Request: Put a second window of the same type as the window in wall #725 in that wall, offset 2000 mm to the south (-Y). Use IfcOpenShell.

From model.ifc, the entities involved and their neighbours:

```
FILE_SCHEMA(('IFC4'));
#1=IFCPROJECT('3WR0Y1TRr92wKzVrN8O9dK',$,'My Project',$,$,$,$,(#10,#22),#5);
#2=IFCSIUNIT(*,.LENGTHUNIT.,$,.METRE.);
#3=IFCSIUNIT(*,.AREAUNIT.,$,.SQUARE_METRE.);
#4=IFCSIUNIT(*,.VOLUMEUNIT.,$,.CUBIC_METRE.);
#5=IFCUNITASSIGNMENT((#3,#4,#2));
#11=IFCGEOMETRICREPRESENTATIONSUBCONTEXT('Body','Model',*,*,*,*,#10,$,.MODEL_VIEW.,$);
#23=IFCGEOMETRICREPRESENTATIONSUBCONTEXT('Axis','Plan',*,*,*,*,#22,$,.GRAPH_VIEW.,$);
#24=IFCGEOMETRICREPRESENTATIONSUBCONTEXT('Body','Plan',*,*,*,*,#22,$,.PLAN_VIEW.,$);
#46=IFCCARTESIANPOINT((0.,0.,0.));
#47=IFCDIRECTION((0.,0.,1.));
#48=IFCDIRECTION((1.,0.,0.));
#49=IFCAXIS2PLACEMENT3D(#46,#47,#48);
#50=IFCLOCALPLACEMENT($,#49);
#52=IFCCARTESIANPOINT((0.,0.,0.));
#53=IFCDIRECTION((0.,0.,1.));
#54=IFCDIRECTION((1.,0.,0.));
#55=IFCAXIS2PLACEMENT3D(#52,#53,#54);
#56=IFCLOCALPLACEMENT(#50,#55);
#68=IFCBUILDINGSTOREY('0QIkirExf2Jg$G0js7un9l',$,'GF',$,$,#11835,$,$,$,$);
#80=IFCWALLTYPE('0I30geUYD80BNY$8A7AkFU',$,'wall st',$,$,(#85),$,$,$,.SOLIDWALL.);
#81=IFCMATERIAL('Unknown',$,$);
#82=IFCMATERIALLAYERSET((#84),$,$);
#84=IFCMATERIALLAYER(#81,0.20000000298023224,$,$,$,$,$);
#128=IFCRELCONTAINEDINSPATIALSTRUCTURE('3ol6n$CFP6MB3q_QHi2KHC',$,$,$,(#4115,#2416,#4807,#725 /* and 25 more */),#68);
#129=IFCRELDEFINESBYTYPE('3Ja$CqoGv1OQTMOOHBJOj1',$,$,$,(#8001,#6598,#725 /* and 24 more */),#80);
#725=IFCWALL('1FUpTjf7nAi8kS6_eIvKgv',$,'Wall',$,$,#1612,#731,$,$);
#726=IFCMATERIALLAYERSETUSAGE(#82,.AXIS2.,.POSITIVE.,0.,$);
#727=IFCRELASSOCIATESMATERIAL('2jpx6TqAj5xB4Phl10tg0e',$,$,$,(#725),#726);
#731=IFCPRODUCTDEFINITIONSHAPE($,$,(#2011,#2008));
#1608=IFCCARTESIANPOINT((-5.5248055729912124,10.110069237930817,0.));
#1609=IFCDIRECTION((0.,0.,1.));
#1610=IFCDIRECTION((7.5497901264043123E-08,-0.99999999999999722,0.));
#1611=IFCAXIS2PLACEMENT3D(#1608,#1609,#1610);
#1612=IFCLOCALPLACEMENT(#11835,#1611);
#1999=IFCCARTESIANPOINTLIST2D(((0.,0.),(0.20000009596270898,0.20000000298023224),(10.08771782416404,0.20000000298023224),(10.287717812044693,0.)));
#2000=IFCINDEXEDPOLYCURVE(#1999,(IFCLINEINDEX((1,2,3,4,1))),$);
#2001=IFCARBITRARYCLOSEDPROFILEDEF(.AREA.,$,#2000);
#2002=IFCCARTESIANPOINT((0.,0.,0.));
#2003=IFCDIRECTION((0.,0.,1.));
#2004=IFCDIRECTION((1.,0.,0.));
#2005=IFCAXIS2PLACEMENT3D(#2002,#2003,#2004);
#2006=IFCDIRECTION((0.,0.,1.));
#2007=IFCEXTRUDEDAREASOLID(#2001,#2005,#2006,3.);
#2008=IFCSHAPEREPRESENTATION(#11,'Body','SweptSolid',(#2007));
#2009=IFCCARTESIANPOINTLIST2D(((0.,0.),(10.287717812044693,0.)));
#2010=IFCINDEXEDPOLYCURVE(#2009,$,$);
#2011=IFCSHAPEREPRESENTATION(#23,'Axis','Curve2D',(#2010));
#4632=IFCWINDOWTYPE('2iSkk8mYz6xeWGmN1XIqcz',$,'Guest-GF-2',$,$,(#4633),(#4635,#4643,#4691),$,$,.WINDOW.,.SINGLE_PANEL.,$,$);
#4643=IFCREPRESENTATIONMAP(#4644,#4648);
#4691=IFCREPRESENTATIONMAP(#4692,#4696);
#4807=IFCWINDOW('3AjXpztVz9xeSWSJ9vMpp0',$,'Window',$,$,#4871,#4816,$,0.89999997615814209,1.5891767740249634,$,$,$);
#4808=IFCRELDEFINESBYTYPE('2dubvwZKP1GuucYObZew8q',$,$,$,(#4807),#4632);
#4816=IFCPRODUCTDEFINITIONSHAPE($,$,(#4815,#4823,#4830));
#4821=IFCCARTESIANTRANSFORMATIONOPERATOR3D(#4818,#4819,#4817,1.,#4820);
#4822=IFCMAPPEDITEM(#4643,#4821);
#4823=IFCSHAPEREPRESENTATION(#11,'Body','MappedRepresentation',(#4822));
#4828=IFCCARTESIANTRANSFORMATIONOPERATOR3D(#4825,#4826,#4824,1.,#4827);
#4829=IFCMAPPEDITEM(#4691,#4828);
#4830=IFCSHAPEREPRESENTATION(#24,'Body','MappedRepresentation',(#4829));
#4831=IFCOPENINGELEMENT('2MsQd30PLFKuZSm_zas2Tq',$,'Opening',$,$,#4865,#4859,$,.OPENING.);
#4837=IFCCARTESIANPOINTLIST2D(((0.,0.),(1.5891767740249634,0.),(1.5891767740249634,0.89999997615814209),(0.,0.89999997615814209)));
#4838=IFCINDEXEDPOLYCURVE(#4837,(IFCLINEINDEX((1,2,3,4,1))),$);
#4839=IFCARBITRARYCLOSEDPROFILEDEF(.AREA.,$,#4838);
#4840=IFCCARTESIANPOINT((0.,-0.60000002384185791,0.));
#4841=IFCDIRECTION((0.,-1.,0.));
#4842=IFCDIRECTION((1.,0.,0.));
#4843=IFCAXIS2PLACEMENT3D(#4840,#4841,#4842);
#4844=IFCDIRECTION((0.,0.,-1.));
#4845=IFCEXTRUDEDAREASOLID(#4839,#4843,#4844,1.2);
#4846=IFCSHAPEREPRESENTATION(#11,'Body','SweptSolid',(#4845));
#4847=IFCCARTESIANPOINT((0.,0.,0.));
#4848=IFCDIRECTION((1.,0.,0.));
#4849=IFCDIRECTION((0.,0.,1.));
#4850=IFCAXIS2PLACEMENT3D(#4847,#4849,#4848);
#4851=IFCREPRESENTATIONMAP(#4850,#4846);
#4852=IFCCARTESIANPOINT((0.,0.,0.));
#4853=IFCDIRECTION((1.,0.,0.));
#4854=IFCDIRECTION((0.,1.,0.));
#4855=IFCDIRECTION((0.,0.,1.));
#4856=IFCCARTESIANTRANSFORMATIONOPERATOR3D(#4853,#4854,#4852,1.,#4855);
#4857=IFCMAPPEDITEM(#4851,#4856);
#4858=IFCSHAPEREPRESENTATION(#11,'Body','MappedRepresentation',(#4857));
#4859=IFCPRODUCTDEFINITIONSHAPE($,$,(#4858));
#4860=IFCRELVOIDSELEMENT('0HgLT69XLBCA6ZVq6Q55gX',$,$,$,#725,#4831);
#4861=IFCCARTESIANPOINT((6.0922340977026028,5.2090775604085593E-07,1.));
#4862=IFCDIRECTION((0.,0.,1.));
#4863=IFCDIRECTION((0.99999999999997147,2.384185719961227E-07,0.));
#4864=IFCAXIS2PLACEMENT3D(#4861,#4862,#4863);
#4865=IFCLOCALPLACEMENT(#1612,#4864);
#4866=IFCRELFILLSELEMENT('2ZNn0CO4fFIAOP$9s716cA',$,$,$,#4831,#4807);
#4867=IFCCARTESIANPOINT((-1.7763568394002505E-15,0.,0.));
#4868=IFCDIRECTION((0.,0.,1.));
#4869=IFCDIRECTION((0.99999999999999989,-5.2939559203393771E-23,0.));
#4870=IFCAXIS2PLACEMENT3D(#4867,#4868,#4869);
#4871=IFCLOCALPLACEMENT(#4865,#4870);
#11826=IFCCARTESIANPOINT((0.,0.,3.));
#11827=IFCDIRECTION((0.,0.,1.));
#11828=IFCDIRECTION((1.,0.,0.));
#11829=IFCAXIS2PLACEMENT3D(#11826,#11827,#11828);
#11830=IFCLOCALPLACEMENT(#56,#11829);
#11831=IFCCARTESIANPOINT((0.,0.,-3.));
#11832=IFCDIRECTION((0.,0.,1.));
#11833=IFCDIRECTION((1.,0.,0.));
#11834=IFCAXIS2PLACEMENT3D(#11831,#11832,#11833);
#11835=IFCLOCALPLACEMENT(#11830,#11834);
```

```python
import ifcopenshell
import ifcopenshell.api.feature
import ifcopenshell.api.geometry
import ifcopenshell.api.root
import ifcopenshell.geom
import ifcopenshell.util.element
import ifcopenshell.util.placement
import ifcopenshell.util.shape
import ifcopenshell.util.unit

model = ifcopenshell.open("model.ifc")
unit_scale = ifcopenshell.util.unit.calculate_unit_scale(model)
settings = ifcopenshell.geom.settings()


def volume(element):
    """Net volume in cubic metres, openings subtracted."""
    shape = ifcopenshell.geom.create_shape(settings, element)
    return ifcopenshell.util.shape.get_volume(shape.geometry)


window = model.by_guid("3AjXpztVz9xeSWSJ9vMpp0")
opening = window.FillsVoids[0].RelatingOpeningElement
wall = opening.VoidsElements[0].RelatingBuildingElement
before = volume(wall)
shift = ifcopenshell.util.placement.get_local_placement(wall.ObjectPlacement)[:3, 0] * 2 / unit_scale

# copy_class copies the void relationship, type, container and properties, but no geometry.
new_opening = ifcopenshell.api.root.copy_class(model, product=opening)
new_opening.Representation = ifcopenshell.util.element.copy_deep(
    model, opening.Representation, exclude=["IfcGeometricRepresentationContext", "IfcRepresentationMap"]
)
new_window = ifcopenshell.api.root.copy_class(model, product=window)
new_window.Representation = ifcopenshell.util.element.copy_deep(
    model, window.Representation, exclude=["IfcGeometricRepresentationContext", "IfcRepresentationMap"]
)
ifcopenshell.api.feature.add_filling(model, opening=new_opening, element=new_window)

for old, new in ((opening, new_opening), (window, new_window)):
    matrix = ifcopenshell.util.placement.get_local_placement(old.ObjectPlacement)
    matrix[:3, 3] += shift
    ifcopenshell.api.geometry.edit_object_placement(model, product=new, matrix=matrix, is_si=False)

after = volume(wall)

print(f"wall volume {before:.3f} -> {after:.3f} m3")

model.write("model_v2.ifc")
```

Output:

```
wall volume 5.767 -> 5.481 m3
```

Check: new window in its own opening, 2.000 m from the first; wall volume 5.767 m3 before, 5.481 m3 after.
